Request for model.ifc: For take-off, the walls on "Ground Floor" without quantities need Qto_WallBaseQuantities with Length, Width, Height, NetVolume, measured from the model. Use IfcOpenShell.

First a look at what the model holds.

```python
import ifcopenshell
import ifcopenshell.util.element
import ifcopenshell.util.unit

model = ifcopenshell.open("model.ifc")
print(model.schema)
for unit_type in ("LENGTHUNIT", "AREAUNIT", "VOLUMEUNIT"):
    print(unit_type, ifcopenshell.util.unit.calculate_unit_scale(model, unit_type))
storey = next(s for s in model.by_type("IfcBuildingStorey") if s.Name == "Ground Floor")
walls = [e for e in ifcopenshell.util.element.get_decomposition(storey) if e.is_a("IfcWall")]
for e in sorted(walls, key=lambda e: e.id()):
    print(e.id(), e.is_a(), e.Name, list(ifcopenshell.util.element.get_psets(e, qtos_only=True)), sep=" | ")
```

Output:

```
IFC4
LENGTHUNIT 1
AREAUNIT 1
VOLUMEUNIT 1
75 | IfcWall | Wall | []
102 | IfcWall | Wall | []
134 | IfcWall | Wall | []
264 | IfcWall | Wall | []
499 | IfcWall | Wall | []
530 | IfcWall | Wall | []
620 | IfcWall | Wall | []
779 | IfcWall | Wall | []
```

```python
import ifcopenshell
import ifcopenshell.api.pset
import ifcopenshell.geom
import ifcopenshell.util.element
import ifcopenshell.util.shape
import ifcopenshell.util.unit

model = ifcopenshell.open("model.ifc")
unit_scale = ifcopenshell.util.unit.calculate_unit_scale(model)
volume_scale = ifcopenshell.util.unit.calculate_unit_scale(model, "VOLUMEUNIT")
settings = ifcopenshell.geom.settings()

storey = next(s for s in model.by_type("IfcBuildingStorey") if s.Name == "Ground Floor")
walls = [e for e in ifcopenshell.util.element.get_decomposition(storey) if e.is_a("IfcWall")]

for e in sorted(walls, key=lambda e: e.id()):
    if ifcopenshell.util.element.get_psets(e, qtos_only=True, should_inherit=False):
        continue
    # Geometry comes back in metres, in the element's own axes.
    shape = ifcopenshell.geom.create_shape(settings, e)
    values = {
        "Length": ifcopenshell.util.shape.get_x(shape.geometry) / unit_scale,
        "Width": ifcopenshell.util.shape.get_y(shape.geometry) / unit_scale,
        "Height": ifcopenshell.util.shape.get_z(shape.geometry) / unit_scale,
        "NetVolume": ifcopenshell.util.shape.get_volume(shape.geometry) / volume_scale,
    }
    qto = ifcopenshell.api.pset.add_qto(model, product=e, name="Qto_WallBaseQuantities")
    ifcopenshell.api.pset.edit_qto(model, qto=qto, properties=values)
    print(e.id(), {k: round(v, 3) for k, v in values.items()})

model.write("model_rev.ifc")
```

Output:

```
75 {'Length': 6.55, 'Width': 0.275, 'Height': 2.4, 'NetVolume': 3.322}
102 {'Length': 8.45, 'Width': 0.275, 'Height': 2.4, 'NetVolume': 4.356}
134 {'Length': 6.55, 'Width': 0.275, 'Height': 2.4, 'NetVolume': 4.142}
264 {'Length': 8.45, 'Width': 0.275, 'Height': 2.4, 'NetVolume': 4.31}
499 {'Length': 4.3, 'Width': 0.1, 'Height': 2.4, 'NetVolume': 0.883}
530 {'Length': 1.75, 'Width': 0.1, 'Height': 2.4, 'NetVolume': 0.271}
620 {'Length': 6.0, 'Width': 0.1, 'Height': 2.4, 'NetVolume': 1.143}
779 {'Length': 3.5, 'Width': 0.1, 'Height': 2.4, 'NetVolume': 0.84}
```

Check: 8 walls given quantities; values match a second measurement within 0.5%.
